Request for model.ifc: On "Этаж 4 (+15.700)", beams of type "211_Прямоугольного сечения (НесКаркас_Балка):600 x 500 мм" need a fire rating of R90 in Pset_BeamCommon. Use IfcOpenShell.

First a look at what the model holds.

```python
import ifcopenshell
import ifcopenshell.util.element

model = ifcopenshell.open("model.ifc")
print(model.schema)
storey = next(s for s in model.by_type("IfcBuildingStorey") if s.Name == "Этаж 4 (+15.700)")
beams = [e for e in ifcopenshell.util.element.get_decomposition(storey) if e.is_a("IfcBeam")]
seen = {}
for e in beams:
    element_type = ifcopenshell.util.element.get_type(e)
    key = (element_type.Name if element_type != e and element_type else None, ifcopenshell.util.element.get_pset(e, "Pset_BeamCommon", "FireRating"))
    seen[key] = seen.get(key, 0) + 1
for (name, value), count in sorted(seen.items(), key=str):
    print(count, "x", name, "|", value)
```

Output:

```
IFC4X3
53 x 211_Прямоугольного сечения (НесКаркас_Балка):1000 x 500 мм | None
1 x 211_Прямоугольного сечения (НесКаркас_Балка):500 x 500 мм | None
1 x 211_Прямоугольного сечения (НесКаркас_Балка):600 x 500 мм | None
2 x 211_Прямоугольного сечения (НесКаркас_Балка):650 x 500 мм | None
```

```python
import ifcopenshell
import ifcopenshell.api.pset
import ifcopenshell.util.element

model = ifcopenshell.open("model.ifc")

storey = next(s for s in model.by_type("IfcBuildingStorey") if s.Name == "Этаж 4 (+15.700)")
beams = [e for e in ifcopenshell.util.element.get_decomposition(storey) if e.is_a("IfcBeam")]

count = 0
for e in beams:
    element_type = ifcopenshell.util.element.get_type(e)
    if element_type in (None, e) or element_type.Name != "211_Прямоугольного сечения (НесКаркас_Балка):600 x 500 мм":
        continue
    # add_pset returns the element's existing set when there is one.
    pset = ifcopenshell.api.pset.add_pset(model, product=e, name="Pset_BeamCommon")
    ifcopenshell.api.pset.edit_pset(model, pset=pset, properties={"FireRating": "R90"})
    count += 1

print(count, "beams updated")

model.write("model-out.ifc")
```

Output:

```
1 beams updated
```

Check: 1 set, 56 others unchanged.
